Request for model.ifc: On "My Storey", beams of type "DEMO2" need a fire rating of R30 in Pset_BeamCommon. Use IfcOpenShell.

First a look at what the model holds.

```python
import ifcopenshell
import ifcopenshell.util.element

model = ifcopenshell.open("model.ifc")
print(model.schema)
storey = next(s for s in model.by_type("IfcBuildingStorey") if s.Name == "My Storey")
beams = [e for e in ifcopenshell.util.element.get_decomposition(storey) if e.is_a("IfcBeam")]
seen = {}
for e in beams:
    element_type = ifcopenshell.util.element.get_type(e)
    key = (element_type.Name if element_type != e and element_type else None, ifcopenshell.util.element.get_pset(e, "Pset_BeamCommon", "FireRating"))
    seen[key] = seen.get(key, 0) + 1
for (name, value), count in sorted(seen.items(), key=str):
    print(count, "x", name, "|", value)
```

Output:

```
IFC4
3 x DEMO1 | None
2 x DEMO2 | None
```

```python
import ifcopenshell
import ifcopenshell.api.pset
import ifcopenshell.util.element

model = ifcopenshell.open("model.ifc")

storey = next(s for s in model.by_type("IfcBuildingStorey") if s.Name == "My Storey")
beams = [e for e in ifcopenshell.util.element.get_decomposition(storey) if e.is_a("IfcBeam")]

count = 0
for e in beams:
    element_type = ifcopenshell.util.element.get_type(e)
    if element_type in (None, e) or element_type.Name != "DEMO2":
        continue
    # add_pset returns the element's existing set when there is one.
    pset = ifcopenshell.api.pset.add_pset(model, product=e, name="Pset_BeamCommon")
    ifcopenshell.api.pset.edit_pset(model, pset=pset, properties={"FireRating": "R30"})
    count += 1

print(count, "beams updated")

model.write("model_rev.ifc")
```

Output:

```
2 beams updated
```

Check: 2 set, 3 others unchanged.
